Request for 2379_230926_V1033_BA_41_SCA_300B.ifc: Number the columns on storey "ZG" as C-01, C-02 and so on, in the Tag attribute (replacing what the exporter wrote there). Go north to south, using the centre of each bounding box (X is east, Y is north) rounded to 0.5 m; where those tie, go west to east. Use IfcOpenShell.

First a look at what the model holds.

```python
import ifcopenshell
import ifcopenshell.util.element
import ifcopenshell.util.placement

model = ifcopenshell.open("2379_230926_V1033_BA_41_SCA_300B.ifc")
print(model.schema)
storey = next(s for s in model.by_type("IfcBuildingStorey") if s.Name == "ZG")
columns = [e for e in ifcopenshell.util.element.get_decomposition(storey) if e.is_a("IfcColumn")]
for e in sorted(columns, key=lambda e: e.id()):
    origin = ifcopenshell.util.placement.get_local_placement(e.ObjectPlacement)[:3, 3]
    print(e.id(), e.Tag, e.Name, origin.round(2) + 0.0, sep=" | ")
```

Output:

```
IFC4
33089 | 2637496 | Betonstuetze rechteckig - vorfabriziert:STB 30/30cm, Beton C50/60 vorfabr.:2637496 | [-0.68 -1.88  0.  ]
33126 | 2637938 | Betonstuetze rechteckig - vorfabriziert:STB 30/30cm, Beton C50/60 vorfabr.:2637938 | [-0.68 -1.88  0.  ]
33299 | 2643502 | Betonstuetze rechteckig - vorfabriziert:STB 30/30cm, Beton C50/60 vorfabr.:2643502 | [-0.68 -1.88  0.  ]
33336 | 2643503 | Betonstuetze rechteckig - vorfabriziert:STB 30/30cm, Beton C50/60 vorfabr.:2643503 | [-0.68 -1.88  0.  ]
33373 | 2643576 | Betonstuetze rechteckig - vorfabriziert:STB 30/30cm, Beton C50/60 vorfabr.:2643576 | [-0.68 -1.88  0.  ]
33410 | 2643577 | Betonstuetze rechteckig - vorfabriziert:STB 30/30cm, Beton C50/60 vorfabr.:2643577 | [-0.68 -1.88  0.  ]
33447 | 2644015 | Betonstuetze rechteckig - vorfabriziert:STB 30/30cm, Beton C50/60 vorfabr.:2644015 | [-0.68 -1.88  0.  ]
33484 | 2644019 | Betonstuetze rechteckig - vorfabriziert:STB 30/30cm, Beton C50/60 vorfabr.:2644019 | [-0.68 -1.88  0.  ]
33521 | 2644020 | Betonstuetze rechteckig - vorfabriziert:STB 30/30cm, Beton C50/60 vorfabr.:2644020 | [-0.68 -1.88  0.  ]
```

```python
import ifcopenshell
import ifcopenshell.geom
import ifcopenshell.util.element
import ifcopenshell.util.shape

model = ifcopenshell.open("2379_230926_V1033_BA_41_SCA_300B.ifc")
settings = ifcopenshell.geom.settings()
settings.set("use-world-coords", True)


def centre(element):
    shape = ifcopenshell.geom.create_shape(settings, element)
    return ifcopenshell.util.shape.get_bbox_centroid(shape.geometry)


storey = next(s for s in model.by_type("IfcBuildingStorey") if s.Name == "ZG")
columns = [e for e in ifcopenshell.util.element.get_decomposition(storey) if e.is_a("IfcColumn")]

# Insertion points can sit at a corner or the storey origin, so sort by the geometry (in metres).
centres = {e: centre(e) for e in columns}
columns.sort(key=lambda e: (-round(centres[e][1] / 0.5), centres[e][0]))

for i, e in enumerate(columns, start=1):
    number = f"C-{i:02d}"
    e.Tag = number
    print(e.id(), number)

model.write("2379_230926_V1033_BA_41_SCA_300B_rev.ifc")
```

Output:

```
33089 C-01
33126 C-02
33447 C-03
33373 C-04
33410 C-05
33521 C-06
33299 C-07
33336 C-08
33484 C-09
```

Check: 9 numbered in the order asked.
